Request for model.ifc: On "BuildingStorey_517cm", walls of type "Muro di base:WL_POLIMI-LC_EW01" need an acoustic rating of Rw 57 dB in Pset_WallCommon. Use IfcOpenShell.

First a look at what the model holds.

```python
import ifcopenshell
import ifcopenshell.util.element

model = ifcopenshell.open("model.ifc")
print(model.schema)
storey = next(s for s in model.by_type("IfcBuildingStorey") if s.Name == "BuildingStorey_517cm")
walls = [e for e in ifcopenshell.util.element.get_decomposition(storey) if e.is_a("IfcWall")]
seen = {}
for e in walls:
    element_type = ifcopenshell.util.element.get_type(e)
    key = (element_type.Name if element_type != e and element_type else None, ifcopenshell.util.element.get_pset(e, "Pset_WallCommon", "AcousticRating"))
    seen[key] = seen.get(key, 0) + 1
for (name, value), count in sorted(seen.items(), key=str):
    print(count, "x", name, "|", value)
```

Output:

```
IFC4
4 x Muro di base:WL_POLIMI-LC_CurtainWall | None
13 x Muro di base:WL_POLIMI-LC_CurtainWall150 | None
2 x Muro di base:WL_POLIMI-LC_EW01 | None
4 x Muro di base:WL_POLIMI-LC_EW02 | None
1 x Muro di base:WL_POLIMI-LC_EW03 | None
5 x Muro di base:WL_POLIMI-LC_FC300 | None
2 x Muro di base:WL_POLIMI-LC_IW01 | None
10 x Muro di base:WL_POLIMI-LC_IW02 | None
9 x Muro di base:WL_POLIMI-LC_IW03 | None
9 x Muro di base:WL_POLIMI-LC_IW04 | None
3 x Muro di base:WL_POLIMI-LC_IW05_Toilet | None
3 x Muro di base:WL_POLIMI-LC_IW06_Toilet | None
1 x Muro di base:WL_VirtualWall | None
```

```python
import ifcopenshell
import ifcopenshell.api.pset
import ifcopenshell.util.element

model = ifcopenshell.open("model.ifc")

storey = next(s for s in model.by_type("IfcBuildingStorey") if s.Name == "BuildingStorey_517cm")
walls = [e for e in ifcopenshell.util.element.get_decomposition(storey) if e.is_a("IfcWall")]

count = 0
for e in walls:
    element_type = ifcopenshell.util.element.get_type(e)
    if element_type in (None, e) or element_type.Name != "Muro di base:WL_POLIMI-LC_EW01":
        continue
    # add_pset returns the element's existing set when there is one.
    pset = ifcopenshell.api.pset.add_pset(model, product=e, name="Pset_WallCommon")
    ifcopenshell.api.pset.edit_pset(model, pset=pset, properties={"AcousticRating": "Rw 57 dB"})
    count += 1

print(count, "walls updated")

model.write("model_rev.ifc")
```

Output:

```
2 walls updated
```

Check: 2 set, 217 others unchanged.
